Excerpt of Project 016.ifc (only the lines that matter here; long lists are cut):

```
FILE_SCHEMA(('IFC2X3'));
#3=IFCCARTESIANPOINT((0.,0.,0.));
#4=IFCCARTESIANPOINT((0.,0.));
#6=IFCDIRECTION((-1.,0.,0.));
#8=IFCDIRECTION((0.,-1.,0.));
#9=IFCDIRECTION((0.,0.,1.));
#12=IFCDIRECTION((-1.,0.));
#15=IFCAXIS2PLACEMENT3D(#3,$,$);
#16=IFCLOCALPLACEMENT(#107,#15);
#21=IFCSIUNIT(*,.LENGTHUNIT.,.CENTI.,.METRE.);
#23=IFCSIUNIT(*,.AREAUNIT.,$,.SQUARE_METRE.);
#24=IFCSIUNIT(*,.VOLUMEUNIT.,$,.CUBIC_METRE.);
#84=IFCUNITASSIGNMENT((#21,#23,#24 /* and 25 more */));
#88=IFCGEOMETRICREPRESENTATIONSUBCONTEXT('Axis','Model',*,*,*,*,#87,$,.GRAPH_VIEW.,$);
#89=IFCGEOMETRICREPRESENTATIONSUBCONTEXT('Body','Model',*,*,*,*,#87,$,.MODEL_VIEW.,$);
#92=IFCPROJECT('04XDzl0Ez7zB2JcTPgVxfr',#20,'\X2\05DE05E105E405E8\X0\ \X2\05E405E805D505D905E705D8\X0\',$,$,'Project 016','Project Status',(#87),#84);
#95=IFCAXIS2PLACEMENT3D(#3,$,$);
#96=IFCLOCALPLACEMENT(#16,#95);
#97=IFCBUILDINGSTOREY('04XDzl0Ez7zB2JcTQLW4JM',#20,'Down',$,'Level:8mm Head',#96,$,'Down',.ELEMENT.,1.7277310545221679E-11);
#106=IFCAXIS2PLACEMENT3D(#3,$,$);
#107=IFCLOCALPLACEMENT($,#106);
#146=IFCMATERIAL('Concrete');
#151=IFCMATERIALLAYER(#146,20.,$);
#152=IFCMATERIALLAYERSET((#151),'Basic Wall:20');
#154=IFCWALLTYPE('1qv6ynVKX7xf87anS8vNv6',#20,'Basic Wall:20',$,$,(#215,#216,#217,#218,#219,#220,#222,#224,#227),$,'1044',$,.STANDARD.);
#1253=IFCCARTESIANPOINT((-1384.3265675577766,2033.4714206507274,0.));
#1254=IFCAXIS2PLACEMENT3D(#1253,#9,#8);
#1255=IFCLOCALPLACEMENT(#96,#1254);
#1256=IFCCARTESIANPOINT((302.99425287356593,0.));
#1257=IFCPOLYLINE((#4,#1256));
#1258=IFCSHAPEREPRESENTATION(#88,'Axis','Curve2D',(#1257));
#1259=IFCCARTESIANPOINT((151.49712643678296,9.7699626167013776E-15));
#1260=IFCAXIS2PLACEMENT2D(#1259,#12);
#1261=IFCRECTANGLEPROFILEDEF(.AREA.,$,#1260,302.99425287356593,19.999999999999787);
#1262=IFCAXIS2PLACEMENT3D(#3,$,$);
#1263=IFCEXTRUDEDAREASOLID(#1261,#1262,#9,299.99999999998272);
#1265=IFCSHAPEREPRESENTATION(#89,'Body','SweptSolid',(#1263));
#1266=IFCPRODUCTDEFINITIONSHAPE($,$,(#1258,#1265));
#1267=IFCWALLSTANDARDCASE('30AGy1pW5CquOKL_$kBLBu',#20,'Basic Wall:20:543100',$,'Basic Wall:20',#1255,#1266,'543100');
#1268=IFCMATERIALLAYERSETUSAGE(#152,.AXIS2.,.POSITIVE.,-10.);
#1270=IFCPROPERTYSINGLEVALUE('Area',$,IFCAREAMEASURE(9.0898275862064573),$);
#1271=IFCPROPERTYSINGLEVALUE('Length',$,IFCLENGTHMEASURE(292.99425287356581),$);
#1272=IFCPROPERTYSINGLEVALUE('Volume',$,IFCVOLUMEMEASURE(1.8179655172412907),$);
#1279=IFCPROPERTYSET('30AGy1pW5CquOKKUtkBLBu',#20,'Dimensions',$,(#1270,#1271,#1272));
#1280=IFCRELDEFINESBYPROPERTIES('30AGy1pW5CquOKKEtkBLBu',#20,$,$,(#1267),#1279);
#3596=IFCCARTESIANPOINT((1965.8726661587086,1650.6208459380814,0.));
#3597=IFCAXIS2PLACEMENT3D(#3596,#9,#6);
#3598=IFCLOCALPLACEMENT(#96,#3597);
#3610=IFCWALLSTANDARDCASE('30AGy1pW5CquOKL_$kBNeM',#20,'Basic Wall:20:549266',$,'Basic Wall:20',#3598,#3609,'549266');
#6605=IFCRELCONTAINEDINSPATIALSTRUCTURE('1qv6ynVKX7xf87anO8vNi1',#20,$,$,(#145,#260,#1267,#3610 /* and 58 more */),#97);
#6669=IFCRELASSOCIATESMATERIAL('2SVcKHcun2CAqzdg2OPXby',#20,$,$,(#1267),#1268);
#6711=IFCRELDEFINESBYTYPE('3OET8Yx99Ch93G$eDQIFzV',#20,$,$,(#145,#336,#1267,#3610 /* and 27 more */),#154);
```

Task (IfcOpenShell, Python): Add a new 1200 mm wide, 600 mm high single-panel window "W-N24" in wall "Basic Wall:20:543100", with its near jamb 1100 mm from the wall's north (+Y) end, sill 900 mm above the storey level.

```python
import numpy as np
import ifcopenshell
import ifcopenshell.api.feature
import ifcopenshell.api.geometry
import ifcopenshell.api.pset
import ifcopenshell.api.root
import ifcopenshell.api.spatial
import ifcopenshell.api.type
import ifcopenshell.geom
import ifcopenshell.util.element
import ifcopenshell.util.placement
import ifcopenshell.util.representation
import ifcopenshell.util.shape
import ifcopenshell.util.unit

model = ifcopenshell.open("Project 016.ifc")
unit_scale = ifcopenshell.util.unit.calculate_unit_scale(model)
area_scale = ifcopenshell.util.unit.calculate_unit_scale(model, "AREAUNIT")
volume_scale = ifcopenshell.util.unit.calculate_unit_scale(model, "VOLUMEUNIT")
settings = ifcopenshell.geom.settings()


def volume(element):
    """Net volume in cubic metres, openings subtracted."""
    shape = ifcopenshell.geom.create_shape(settings, element)
    return ifcopenshell.util.shape.get_volume(shape.geometry)


wall = model.by_id(1267)
storey = ifcopenshell.util.element.get_container(wall, ifc_class="IfcBuildingStorey")
context = ifcopenshell.util.representation.get_context(model, "Model", "Body", "MODEL_VIEW")
before = volume(wall)

width, height, from_end, sill = 1.2, 0.6, 1.1, 0.9  # metres

# The wall runs along its own X axis, and the end named is its -X end.
wall_shape = ifcopenshell.geom.create_shape(settings, wall)
x, y, z = ifcopenshell.util.shape.get_vertices(wall_shape.geometry).T
start = x.min() + from_end
face, thickness = float(y.min()), float(y.max() - y.min())
wall_matrix = ifcopenshell.util.placement.get_local_placement(wall.ObjectPlacement)
level = ifcopenshell.util.placement.get_local_placement(storey.ObjectPlacement)[2, 3]


def in_wall(x, y):
    """Placement at x, y metres in the wall's axes, at sill height."""
    matrix = wall_matrix.copy()
    matrix[:, 3] = wall_matrix @ np.array([x / unit_scale, y / unit_scale, 0.0, 1.0])
    matrix[2, 3] = level + sill / unit_scale
    return matrix


# Opening: a box that overshoots both wall faces by 50 mm.
opening = ifcopenshell.api.root.create_entity(model, ifc_class="IfcOpeningElement")
box = ifcopenshell.api.geometry.add_wall_representation(
    model, context=context, length=width, height=height, thickness=thickness + 0.1
)
ifcopenshell.api.geometry.assign_representation(model, product=opening, representation=box)
ifcopenshell.api.geometry.edit_object_placement(model, product=opening, matrix=in_wall(start, face - 0.05), is_si=False)
ifcopenshell.api.feature.add_feature(model, feature=opening, element=wall)

window = ifcopenshell.api.root.create_entity(model, ifc_class="IfcWindow", name="W-N24")
window.OverallWidth, window.OverallHeight = width / unit_scale, height / unit_scale
body = ifcopenshell.api.geometry.add_window_representation(
    model,
    context=context,
    overall_width=window.OverallWidth,
    overall_height=window.OverallHeight,
    partition_type="SINGLE_PANEL",
)
ifcopenshell.api.geometry.assign_representation(model, product=window, representation=body)
ifcopenshell.api.spatial.assign_container(model, products=[window], relating_structure=storey)
fills = ifcopenshell.api.feature.add_filling(model, opening=opening, element=window)
fills.OwnerHistory = window.OwnerHistory  # required in IFC2X3

# IFC2X3 keeps the operation on the window style.
style = ifcopenshell.api.root.create_entity(model, ifc_class="IfcWindowStyle", name="W-N24")
style.OperationType, style.ConstructionType = "SINGLE_PANEL", "NOTDEFINED"
style.ParameterTakesPrecedence = style.Sizeable = False
ifcopenshell.api.type.assign_type(model, related_objects=[window], relating_type=style)

# Centre the window in the wall's thickness.
ifcopenshell.api.geometry.edit_object_placement(model, product=window, matrix=in_wall(start, face), is_si=False)
window_shape = ifcopenshell.geom.create_shape(settings, window)
depth = ifcopenshell.util.shape.get_vertices(window_shape.geometry)[:, 1]
offset = face + thickness / 2 - (depth.min() + depth.max()) / 2
ifcopenshell.api.geometry.edit_object_placement(model, product=window, matrix=in_wall(start, offset), is_si=False)

after = volume(wall)

# Update the wall's stored quantities.
pset = model.by_id(ifcopenshell.util.element.get_pset(wall, "Dimensions", should_inherit=False)["id"])
ifcopenshell.api.pset.edit_pset(model, pset=pset, properties={
    "Area": model.create_entity("IfcAreaMeasure", after / thickness / area_scale),
    "Volume": model.create_entity("IfcVolumeMeasure", after / volume_scale),
})

print(f"wall volume {before:.3f} -> {after:.3f} m3")

model.write("Project 016_v2.ifc")
```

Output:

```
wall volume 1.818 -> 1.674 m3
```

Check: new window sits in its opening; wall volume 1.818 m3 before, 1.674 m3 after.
